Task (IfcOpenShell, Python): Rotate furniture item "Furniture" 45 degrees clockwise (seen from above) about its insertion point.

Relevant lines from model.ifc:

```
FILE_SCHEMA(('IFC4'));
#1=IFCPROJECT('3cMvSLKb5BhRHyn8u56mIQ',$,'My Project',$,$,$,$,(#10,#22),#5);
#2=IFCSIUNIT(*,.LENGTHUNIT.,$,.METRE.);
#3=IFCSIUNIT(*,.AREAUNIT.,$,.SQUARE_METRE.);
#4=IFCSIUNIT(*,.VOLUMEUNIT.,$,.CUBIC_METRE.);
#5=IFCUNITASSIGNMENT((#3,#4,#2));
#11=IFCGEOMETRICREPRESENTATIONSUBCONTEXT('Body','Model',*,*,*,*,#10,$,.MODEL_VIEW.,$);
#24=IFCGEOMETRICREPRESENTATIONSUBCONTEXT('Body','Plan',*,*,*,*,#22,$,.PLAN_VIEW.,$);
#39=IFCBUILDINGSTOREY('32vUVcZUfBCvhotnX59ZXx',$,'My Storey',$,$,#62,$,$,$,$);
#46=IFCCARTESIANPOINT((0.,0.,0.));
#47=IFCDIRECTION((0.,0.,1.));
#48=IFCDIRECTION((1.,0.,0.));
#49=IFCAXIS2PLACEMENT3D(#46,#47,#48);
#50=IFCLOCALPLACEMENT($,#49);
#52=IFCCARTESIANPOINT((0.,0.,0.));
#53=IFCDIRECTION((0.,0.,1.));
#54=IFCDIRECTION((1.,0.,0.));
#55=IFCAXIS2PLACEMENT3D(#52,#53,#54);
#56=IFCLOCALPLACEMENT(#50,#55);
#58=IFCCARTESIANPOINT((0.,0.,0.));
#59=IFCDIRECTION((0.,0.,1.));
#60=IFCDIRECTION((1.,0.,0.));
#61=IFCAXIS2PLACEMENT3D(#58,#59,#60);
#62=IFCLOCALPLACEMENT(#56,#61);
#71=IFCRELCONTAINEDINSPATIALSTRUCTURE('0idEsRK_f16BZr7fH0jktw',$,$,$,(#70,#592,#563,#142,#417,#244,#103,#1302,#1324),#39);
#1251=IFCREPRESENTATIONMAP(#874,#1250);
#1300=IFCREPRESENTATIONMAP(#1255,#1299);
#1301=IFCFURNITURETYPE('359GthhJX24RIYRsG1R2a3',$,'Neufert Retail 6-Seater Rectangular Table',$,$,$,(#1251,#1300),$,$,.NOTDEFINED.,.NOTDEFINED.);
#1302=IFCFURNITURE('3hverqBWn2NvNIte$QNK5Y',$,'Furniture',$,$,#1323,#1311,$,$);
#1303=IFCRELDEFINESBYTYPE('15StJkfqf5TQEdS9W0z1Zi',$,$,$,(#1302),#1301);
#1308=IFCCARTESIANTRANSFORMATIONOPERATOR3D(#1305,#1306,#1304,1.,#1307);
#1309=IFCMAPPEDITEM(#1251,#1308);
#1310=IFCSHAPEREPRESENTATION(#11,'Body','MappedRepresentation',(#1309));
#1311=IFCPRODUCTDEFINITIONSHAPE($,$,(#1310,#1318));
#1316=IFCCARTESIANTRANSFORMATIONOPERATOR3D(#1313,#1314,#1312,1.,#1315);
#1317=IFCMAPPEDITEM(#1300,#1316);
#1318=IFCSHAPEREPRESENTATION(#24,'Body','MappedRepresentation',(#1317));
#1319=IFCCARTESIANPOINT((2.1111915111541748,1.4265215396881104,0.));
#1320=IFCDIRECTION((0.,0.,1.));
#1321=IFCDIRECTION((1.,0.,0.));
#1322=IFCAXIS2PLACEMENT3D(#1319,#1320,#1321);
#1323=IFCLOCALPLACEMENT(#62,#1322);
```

```python
import ifcopenshell
import ifcopenshell.api.geometry
import ifcopenshell.util.placement

model = ifcopenshell.open("model.ifc")

item = model.by_guid("3hverqBWn2NvNIte$QNK5Y")
matrix = ifcopenshell.util.placement.get_local_placement(item.ObjectPlacement)
matrix = matrix @ ifcopenshell.util.placement.rotation(-45, "Z")
ifcopenshell.api.geometry.edit_object_placement(model, product=item, matrix=matrix, is_si=False)

print(ifcopenshell.util.placement.get_local_placement(item.ObjectPlacement).round(3) + 0.0)

model.write("model_updated.ifc")
```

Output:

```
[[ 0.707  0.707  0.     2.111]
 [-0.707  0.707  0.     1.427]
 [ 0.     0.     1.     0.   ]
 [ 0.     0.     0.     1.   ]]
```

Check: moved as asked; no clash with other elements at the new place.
